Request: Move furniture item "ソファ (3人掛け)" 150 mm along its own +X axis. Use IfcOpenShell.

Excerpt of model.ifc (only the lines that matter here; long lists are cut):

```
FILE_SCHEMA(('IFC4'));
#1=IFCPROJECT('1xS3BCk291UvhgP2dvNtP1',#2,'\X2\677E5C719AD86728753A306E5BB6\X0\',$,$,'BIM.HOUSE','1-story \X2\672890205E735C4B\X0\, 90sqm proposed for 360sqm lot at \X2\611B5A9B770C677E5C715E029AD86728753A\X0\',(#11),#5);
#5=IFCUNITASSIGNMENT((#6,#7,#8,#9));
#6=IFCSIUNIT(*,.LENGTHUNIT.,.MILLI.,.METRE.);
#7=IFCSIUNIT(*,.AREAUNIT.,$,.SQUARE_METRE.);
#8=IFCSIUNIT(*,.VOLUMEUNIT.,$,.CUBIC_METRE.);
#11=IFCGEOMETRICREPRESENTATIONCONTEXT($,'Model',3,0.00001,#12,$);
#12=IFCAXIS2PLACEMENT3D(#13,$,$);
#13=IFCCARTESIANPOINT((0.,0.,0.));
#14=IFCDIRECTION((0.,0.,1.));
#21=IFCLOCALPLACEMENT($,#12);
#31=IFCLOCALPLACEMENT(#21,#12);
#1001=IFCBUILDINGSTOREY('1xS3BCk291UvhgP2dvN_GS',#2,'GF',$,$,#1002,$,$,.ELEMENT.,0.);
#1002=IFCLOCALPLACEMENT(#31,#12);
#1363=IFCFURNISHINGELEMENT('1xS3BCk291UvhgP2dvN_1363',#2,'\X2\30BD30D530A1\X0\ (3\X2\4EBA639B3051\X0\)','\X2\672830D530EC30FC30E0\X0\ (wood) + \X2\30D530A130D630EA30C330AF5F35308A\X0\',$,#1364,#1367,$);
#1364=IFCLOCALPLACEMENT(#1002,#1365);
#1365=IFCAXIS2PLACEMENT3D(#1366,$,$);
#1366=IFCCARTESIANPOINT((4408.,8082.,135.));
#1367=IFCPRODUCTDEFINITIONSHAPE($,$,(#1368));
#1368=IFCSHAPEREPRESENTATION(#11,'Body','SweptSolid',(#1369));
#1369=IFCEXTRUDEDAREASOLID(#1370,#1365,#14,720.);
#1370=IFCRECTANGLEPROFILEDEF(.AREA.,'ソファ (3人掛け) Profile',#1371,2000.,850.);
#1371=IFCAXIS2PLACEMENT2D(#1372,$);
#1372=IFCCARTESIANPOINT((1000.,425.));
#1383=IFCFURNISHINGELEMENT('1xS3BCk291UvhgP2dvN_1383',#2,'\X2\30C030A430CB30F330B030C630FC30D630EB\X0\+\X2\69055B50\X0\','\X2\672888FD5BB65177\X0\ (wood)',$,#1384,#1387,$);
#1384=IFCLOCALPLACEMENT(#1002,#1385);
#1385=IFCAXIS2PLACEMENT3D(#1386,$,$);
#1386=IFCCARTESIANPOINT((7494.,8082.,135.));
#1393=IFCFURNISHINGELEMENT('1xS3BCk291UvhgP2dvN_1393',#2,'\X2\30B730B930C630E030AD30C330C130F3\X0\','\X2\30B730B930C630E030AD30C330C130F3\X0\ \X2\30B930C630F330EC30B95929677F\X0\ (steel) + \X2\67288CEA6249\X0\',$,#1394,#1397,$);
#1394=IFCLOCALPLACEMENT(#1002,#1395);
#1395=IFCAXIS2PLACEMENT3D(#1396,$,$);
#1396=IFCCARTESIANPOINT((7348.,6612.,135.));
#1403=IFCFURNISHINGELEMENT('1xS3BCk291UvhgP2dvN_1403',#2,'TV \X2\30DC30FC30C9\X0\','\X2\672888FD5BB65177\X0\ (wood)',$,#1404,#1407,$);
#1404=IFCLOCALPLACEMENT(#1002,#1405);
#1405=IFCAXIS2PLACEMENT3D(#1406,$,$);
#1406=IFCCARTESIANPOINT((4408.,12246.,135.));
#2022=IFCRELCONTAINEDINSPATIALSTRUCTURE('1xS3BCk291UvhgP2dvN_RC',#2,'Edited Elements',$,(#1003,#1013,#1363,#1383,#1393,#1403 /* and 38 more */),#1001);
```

```python
import ifcopenshell
import ifcopenshell.api.geometry
import ifcopenshell.util.placement

model = ifcopenshell.open("model.ifc")

item = model.by_guid("1xS3BCk291UvhgP2dvN_1363")
matrix = ifcopenshell.util.placement.get_local_placement(item.ObjectPlacement)
matrix[:3, 3] += matrix[:3, 0] * 150.0
ifcopenshell.api.geometry.edit_object_placement(model, product=item, matrix=matrix, is_si=False)

print(ifcopenshell.util.placement.get_local_placement(item.ObjectPlacement).round(3) + 0.0)

model.write("model_edited.ifc")
```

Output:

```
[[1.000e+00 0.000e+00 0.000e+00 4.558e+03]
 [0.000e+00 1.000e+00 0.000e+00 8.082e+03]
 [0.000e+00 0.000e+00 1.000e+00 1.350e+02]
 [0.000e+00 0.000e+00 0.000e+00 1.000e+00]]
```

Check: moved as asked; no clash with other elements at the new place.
